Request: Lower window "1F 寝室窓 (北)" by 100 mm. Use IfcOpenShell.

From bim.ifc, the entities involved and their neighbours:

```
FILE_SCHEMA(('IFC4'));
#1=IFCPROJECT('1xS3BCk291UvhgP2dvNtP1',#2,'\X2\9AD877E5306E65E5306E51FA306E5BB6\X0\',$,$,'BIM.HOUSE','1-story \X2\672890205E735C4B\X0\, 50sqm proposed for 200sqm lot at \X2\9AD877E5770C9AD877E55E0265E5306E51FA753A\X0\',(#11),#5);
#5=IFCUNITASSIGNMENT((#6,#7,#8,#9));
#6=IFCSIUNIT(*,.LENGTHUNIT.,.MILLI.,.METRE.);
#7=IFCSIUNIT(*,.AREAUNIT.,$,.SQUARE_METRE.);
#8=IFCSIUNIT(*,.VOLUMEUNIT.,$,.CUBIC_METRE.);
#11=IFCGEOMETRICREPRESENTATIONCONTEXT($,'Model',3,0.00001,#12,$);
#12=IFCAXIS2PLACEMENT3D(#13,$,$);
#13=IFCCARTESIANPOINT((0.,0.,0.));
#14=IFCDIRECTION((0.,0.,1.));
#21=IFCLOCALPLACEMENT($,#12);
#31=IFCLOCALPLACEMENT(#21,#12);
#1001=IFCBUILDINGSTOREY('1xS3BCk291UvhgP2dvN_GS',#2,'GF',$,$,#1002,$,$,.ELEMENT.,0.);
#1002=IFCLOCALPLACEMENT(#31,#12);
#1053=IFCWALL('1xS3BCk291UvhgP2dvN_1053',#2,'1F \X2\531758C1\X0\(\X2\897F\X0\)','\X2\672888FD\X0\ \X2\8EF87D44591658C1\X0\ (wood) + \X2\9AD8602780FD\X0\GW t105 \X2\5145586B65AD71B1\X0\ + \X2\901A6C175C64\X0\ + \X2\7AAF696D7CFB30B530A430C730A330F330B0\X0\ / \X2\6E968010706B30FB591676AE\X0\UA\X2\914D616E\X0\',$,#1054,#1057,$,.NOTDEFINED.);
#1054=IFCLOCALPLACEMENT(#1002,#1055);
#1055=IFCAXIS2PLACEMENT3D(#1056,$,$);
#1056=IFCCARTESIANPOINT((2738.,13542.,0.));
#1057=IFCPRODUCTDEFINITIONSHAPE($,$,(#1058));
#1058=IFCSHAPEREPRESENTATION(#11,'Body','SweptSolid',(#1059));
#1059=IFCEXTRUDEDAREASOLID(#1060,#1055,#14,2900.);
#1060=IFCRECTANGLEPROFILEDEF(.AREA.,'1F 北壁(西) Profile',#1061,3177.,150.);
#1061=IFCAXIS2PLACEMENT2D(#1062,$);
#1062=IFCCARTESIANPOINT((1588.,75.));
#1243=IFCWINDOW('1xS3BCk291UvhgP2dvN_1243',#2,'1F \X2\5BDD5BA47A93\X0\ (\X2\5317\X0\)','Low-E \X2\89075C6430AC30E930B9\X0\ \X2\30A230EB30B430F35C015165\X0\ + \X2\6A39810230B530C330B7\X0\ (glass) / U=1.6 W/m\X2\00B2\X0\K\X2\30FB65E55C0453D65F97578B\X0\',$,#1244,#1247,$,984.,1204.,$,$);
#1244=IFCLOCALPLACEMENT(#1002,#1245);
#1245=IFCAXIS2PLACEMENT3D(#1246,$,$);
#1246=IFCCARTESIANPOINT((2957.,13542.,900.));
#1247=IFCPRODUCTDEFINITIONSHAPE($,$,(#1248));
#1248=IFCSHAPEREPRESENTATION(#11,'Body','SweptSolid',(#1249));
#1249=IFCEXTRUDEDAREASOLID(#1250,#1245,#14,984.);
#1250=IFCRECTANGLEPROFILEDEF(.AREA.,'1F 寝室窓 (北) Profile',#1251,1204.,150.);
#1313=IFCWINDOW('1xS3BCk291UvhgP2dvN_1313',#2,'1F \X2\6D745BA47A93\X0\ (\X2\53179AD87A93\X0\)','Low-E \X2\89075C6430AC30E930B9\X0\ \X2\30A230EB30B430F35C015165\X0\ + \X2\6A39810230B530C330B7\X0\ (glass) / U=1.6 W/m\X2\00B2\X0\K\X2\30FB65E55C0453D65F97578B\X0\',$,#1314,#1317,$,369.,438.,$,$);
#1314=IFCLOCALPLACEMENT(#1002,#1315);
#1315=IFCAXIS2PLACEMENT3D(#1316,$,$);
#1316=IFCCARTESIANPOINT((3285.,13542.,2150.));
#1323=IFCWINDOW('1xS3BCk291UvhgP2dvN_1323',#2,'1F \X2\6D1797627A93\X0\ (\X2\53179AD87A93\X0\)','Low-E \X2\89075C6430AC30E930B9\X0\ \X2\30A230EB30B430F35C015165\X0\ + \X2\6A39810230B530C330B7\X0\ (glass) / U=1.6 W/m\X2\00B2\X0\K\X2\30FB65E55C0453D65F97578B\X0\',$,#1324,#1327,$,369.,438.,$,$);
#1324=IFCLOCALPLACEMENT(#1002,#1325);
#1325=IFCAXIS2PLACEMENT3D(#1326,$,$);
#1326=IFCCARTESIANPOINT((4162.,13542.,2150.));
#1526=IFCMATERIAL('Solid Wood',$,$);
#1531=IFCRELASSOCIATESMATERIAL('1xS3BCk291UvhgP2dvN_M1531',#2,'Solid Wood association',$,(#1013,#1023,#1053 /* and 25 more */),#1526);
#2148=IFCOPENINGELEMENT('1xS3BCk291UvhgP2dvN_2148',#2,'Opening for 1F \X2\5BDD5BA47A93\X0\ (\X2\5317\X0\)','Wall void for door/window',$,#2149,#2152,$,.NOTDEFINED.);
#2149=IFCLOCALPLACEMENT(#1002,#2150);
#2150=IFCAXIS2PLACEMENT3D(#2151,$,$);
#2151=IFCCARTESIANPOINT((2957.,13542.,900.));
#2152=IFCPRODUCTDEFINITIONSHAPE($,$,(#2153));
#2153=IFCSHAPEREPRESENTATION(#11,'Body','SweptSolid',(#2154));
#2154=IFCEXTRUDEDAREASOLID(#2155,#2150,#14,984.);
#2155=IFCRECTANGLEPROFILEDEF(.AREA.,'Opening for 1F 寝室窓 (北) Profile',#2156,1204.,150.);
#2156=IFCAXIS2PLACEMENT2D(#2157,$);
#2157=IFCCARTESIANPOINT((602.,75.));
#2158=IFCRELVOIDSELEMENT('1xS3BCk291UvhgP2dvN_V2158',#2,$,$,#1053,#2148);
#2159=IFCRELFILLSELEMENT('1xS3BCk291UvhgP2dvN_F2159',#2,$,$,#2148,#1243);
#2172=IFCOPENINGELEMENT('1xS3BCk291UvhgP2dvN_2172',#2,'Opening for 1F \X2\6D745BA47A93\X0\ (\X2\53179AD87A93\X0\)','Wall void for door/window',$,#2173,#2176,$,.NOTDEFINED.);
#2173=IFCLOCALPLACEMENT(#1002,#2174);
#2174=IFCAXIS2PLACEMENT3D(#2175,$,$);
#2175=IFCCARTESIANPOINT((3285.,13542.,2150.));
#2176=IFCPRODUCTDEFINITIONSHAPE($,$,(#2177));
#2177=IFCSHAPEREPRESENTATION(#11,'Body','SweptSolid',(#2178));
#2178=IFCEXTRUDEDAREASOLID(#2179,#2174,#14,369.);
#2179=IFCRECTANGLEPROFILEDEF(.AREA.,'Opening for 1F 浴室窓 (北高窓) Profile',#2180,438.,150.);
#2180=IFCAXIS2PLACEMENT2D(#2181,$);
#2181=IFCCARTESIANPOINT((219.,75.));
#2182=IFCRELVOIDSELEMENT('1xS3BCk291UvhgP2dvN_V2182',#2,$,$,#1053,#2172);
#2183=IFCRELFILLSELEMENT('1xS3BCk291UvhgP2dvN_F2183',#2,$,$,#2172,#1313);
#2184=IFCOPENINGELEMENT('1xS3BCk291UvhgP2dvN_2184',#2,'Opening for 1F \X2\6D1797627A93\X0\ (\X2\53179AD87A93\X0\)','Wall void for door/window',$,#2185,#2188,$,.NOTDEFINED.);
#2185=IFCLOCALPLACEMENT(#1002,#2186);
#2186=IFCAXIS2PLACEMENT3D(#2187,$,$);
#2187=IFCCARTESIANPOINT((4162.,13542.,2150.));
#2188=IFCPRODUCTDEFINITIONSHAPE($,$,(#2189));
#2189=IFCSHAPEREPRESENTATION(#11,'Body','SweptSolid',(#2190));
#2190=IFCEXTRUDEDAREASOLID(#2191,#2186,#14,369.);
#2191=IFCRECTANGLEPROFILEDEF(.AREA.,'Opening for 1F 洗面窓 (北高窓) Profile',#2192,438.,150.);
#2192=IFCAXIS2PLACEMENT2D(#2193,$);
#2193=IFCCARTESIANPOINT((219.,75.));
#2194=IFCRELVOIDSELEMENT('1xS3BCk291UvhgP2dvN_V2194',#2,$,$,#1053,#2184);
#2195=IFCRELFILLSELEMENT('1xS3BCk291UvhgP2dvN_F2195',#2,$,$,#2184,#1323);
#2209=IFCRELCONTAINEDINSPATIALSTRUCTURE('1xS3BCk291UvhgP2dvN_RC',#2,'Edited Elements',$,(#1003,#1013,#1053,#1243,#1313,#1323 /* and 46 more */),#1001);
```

```python
import numpy as np
import ifcopenshell
import ifcopenshell.api.geometry
import ifcopenshell.util.placement
import ifcopenshell.util.unit

model = ifcopenshell.open("bim.ifc")
unit_scale = ifcopenshell.util.unit.calculate_unit_scale(model)

window = model.by_guid("1xS3BCk291UvhgP2dvN_1243")
opening = window.FillsVoids[0].RelatingOpeningElement
dz = -100.0

shift = np.array([0.0, 0.0, dz])
# The window is not placed relative to its opening, so move both.
for product in (opening, window):
    matrix = ifcopenshell.util.placement.get_local_placement(product.ObjectPlacement)
    matrix[:3, 3] += shift
    ifcopenshell.api.geometry.edit_object_placement(model, product=product, matrix=matrix, is_si=False)

print(f"moved by {dz * unit_scale:+.3f} m")

model.write("bim_updated.ifc")
```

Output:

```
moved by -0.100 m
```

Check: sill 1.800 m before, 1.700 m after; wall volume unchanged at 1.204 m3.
